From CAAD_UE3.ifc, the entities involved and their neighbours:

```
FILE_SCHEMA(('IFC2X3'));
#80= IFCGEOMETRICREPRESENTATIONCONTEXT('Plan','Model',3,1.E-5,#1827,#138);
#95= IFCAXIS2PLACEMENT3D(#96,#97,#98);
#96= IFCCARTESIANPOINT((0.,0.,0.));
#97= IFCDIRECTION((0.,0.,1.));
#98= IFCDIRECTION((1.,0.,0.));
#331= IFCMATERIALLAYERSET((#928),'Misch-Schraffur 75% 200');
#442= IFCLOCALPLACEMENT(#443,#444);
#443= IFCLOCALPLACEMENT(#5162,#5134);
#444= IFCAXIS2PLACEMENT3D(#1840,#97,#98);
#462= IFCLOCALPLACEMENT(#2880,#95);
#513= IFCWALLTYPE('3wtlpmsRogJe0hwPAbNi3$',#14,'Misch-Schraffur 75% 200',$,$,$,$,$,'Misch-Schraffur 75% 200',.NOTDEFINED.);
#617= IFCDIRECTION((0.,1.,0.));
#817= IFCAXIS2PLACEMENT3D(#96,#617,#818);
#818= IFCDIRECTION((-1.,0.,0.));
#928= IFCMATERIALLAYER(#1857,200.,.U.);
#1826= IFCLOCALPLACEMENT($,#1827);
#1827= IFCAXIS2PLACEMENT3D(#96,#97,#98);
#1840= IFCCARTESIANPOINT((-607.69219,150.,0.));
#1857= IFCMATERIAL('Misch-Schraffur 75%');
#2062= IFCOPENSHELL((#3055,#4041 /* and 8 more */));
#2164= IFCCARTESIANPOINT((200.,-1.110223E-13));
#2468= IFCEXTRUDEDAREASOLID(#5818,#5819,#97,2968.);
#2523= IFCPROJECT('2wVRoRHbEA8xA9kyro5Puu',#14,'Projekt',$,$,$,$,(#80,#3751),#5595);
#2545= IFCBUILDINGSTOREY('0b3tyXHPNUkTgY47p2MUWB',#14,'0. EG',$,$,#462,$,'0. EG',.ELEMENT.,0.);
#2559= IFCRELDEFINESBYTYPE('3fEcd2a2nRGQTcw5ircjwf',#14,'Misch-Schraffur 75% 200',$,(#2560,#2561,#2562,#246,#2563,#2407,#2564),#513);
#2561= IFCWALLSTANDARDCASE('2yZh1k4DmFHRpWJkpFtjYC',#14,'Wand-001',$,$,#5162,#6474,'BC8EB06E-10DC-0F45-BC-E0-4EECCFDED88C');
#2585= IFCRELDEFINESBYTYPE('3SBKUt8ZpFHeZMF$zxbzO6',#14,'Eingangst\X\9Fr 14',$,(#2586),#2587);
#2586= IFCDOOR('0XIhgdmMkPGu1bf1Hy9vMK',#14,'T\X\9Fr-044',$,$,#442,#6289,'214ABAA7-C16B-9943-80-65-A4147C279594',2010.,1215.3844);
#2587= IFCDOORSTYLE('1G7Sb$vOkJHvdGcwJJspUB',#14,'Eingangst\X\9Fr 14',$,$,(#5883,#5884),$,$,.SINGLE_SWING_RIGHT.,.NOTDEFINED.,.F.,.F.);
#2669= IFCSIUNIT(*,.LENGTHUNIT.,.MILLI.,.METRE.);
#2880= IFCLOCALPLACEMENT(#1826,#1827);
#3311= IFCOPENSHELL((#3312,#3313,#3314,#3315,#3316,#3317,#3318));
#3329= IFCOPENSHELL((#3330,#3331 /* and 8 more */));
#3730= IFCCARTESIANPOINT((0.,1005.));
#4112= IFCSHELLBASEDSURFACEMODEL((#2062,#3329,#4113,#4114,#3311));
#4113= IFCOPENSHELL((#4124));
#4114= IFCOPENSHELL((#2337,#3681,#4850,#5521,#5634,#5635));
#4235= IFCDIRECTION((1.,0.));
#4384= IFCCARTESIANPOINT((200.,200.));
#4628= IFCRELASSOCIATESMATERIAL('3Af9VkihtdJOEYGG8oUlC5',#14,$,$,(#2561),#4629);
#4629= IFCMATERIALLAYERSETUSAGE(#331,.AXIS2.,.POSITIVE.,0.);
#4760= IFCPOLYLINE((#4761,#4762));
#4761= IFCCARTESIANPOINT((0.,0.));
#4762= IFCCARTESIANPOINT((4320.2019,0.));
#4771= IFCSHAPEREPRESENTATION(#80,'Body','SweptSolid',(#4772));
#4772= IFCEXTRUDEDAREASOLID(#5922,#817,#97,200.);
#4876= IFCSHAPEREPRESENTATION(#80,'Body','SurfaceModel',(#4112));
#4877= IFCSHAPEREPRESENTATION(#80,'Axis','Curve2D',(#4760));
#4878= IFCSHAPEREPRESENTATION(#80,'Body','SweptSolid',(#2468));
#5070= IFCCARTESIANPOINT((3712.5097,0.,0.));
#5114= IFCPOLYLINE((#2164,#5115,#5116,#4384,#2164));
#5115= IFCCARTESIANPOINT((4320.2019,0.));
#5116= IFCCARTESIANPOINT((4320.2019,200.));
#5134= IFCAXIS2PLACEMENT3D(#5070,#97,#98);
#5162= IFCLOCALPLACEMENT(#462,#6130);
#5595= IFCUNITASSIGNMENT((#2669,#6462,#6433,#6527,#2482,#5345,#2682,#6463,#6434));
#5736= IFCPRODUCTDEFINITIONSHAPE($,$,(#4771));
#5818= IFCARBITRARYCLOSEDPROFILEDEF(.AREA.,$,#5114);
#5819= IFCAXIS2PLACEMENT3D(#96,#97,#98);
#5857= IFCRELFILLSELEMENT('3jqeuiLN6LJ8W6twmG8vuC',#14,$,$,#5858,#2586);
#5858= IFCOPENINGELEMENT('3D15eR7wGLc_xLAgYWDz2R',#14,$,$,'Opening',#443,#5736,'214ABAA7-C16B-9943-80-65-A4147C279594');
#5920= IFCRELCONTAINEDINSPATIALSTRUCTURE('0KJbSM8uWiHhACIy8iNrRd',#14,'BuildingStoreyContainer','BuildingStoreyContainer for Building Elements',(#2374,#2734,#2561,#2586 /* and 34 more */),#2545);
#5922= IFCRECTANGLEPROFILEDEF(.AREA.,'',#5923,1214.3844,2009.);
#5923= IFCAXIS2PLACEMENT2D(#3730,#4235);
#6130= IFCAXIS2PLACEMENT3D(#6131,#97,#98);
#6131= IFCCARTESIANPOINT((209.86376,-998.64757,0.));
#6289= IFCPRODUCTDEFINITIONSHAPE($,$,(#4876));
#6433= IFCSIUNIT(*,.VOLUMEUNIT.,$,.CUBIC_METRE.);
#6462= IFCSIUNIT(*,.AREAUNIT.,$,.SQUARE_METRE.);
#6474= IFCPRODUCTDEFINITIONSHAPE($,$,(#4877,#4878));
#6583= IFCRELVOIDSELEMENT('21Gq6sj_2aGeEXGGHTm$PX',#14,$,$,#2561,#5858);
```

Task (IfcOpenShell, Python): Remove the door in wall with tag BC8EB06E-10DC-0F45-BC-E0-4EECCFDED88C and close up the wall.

```python
import ifcopenshell
import ifcopenshell.api.feature
import ifcopenshell.api.root
import ifcopenshell.geom
import ifcopenshell.util.shape

model = ifcopenshell.open("CAAD_UE3.ifc")
settings = ifcopenshell.geom.settings()


def volume(element):
    """Net volume in cubic metres, openings subtracted."""
    shape = ifcopenshell.geom.create_shape(settings, element)
    return ifcopenshell.util.shape.get_volume(shape.geometry)


door = model.by_id(2586)
opening = door.FillsVoids[0].RelatingOpeningElement
wall = opening.VoidsElements[0].RelatingBuildingElement
before = volume(wall)

ifcopenshell.api.root.remove_product(model, product=door)
ifcopenshell.api.feature.remove_feature(model, feature=opening)

after = volume(wall)

print(f"wall volume {before:.3f} -> {after:.3f} m3")

model.write("CAAD_UE3_edited.ifc")
```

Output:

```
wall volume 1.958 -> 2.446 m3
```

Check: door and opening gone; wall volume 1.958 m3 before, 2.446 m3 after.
